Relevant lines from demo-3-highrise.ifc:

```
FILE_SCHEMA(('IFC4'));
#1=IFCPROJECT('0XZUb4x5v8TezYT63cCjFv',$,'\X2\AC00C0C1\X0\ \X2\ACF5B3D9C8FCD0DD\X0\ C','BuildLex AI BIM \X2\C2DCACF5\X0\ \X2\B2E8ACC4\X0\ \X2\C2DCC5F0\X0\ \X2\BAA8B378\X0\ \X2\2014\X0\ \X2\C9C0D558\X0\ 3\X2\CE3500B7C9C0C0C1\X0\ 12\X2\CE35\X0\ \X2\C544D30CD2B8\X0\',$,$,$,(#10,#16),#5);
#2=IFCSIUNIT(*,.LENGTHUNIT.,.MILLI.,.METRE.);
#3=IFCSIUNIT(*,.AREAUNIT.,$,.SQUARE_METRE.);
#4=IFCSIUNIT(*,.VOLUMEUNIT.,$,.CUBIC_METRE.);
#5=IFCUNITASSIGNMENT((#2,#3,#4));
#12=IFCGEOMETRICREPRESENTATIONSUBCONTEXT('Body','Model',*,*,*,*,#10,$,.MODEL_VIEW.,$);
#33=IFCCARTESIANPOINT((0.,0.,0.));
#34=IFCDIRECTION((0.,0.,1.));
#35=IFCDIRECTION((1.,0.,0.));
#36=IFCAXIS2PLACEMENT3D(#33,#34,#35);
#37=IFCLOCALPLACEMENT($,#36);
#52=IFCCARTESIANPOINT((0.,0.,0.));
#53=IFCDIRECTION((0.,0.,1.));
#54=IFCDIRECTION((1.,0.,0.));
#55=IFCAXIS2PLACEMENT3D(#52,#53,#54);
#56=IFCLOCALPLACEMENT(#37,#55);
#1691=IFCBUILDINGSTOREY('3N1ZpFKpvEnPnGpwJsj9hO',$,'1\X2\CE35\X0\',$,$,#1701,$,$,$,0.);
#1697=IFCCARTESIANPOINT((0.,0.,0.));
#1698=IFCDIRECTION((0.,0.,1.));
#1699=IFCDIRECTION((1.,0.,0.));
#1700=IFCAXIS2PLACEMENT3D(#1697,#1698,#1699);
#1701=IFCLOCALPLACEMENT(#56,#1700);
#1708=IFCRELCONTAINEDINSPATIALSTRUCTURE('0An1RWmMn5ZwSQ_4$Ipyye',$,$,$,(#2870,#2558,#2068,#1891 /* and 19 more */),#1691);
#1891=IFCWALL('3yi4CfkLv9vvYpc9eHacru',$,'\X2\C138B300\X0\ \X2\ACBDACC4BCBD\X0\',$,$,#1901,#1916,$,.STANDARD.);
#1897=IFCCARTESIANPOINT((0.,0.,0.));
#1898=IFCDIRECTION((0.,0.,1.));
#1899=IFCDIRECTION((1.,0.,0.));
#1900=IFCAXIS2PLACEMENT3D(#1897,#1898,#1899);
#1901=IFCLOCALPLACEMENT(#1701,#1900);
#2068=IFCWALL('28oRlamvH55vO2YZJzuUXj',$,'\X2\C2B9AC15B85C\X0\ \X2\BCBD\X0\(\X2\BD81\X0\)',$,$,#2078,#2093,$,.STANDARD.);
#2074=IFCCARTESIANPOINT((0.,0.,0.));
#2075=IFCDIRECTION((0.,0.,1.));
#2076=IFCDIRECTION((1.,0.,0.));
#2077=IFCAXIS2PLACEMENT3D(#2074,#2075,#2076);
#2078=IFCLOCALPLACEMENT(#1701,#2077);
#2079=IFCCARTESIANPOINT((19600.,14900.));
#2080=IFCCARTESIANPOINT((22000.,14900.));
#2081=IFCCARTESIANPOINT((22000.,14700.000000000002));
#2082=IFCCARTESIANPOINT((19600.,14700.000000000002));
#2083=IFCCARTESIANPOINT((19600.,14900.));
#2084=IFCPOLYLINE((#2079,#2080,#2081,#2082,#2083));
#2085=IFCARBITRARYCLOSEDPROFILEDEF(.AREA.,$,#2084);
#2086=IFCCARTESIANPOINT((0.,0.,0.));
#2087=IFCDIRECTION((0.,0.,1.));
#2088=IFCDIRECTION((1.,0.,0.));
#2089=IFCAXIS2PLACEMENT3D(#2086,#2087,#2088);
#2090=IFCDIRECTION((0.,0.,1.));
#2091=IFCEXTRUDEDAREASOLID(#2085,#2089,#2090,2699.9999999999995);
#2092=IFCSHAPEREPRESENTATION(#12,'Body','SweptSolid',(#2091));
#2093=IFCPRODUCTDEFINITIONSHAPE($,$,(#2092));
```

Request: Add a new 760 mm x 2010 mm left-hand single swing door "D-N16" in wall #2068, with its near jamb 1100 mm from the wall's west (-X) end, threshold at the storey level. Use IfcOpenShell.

```python
import numpy as np
import ifcopenshell
import ifcopenshell.api.feature
import ifcopenshell.api.geometry
import ifcopenshell.api.root
import ifcopenshell.api.spatial
import ifcopenshell.geom
import ifcopenshell.util.element
import ifcopenshell.util.placement
import ifcopenshell.util.representation
import ifcopenshell.util.shape
import ifcopenshell.util.unit

model = ifcopenshell.open("demo-3-highrise.ifc")
unit_scale = ifcopenshell.util.unit.calculate_unit_scale(model)
settings = ifcopenshell.geom.settings()


def volume(element):
    """Net volume in cubic metres, openings subtracted."""
    shape = ifcopenshell.geom.create_shape(settings, element)
    return ifcopenshell.util.shape.get_volume(shape.geometry)


wall = model.by_guid("28oRlamvH55vO2YZJzuUXj")
storey = ifcopenshell.util.element.get_container(wall, ifc_class="IfcBuildingStorey")
context = ifcopenshell.util.representation.get_context(model, "Model", "Body", "MODEL_VIEW")
before = volume(wall)

width, height, from_end, sill = 0.76, 2.01, 1.1, 0.0  # metres

# The wall runs along its own X axis, and the end named is its -X end.
wall_shape = ifcopenshell.geom.create_shape(settings, wall)
x, y, z = ifcopenshell.util.shape.get_vertices(wall_shape.geometry).T
start = x.min() + from_end
face, thickness = float(y.min()), float(y.max() - y.min())
wall_matrix = ifcopenshell.util.placement.get_local_placement(wall.ObjectPlacement)
level = ifcopenshell.util.placement.get_local_placement(storey.ObjectPlacement)[2, 3]


def in_wall(x, y):
    """Placement at x, y metres in the wall's axes, at sill height."""
    matrix = wall_matrix.copy()
    matrix[:, 3] = wall_matrix @ np.array([x / unit_scale, y / unit_scale, 0.0, 1.0])
    matrix[2, 3] = level + sill / unit_scale
    return matrix


# Opening: a box that overshoots both wall faces by 50 mm.
opening = ifcopenshell.api.root.create_entity(model, ifc_class="IfcOpeningElement", predefined_type="OPENING")
box = ifcopenshell.api.geometry.add_wall_representation(
    model, context=context, length=width, height=height, thickness=thickness + 0.1
)
ifcopenshell.api.geometry.assign_representation(model, product=opening, representation=box)
ifcopenshell.api.geometry.edit_object_placement(model, product=opening, matrix=in_wall(start, face - 0.05), is_si=False)
ifcopenshell.api.feature.add_feature(model, feature=opening, element=wall)

door = ifcopenshell.api.root.create_entity(model, ifc_class="IfcDoor", name="D-N16", predefined_type="DOOR")
door.OverallWidth, door.OverallHeight = width / unit_scale, height / unit_scale
door.OperationType = "SINGLE_SWING_LEFT"
body = ifcopenshell.api.geometry.add_door_representation(
    model,
    context=context,
    overall_width=door.OverallWidth,
    overall_height=door.OverallHeight,
    operation_type="SINGLE_SWING_LEFT",
    lining_properties={"LiningDepth": thickness / unit_scale, "ThresholdDepth": thickness / unit_scale},
)
ifcopenshell.api.geometry.assign_representation(model, product=door, representation=body)
ifcopenshell.api.spatial.assign_container(model, products=[door], relating_structure=storey)
ifcopenshell.api.feature.add_filling(model, opening=opening, element=door)

# The lining spans the wall, so the door starts at the wall face.
ifcopenshell.api.geometry.edit_object_placement(model, product=door, matrix=in_wall(start, face), is_si=False)

after = volume(wall)

print(f"wall volume {before:.3f} -> {after:.3f} m3")

model.write("demo-3-highrise_v2.ifc")
```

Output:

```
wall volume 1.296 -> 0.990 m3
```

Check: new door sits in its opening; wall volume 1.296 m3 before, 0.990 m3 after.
